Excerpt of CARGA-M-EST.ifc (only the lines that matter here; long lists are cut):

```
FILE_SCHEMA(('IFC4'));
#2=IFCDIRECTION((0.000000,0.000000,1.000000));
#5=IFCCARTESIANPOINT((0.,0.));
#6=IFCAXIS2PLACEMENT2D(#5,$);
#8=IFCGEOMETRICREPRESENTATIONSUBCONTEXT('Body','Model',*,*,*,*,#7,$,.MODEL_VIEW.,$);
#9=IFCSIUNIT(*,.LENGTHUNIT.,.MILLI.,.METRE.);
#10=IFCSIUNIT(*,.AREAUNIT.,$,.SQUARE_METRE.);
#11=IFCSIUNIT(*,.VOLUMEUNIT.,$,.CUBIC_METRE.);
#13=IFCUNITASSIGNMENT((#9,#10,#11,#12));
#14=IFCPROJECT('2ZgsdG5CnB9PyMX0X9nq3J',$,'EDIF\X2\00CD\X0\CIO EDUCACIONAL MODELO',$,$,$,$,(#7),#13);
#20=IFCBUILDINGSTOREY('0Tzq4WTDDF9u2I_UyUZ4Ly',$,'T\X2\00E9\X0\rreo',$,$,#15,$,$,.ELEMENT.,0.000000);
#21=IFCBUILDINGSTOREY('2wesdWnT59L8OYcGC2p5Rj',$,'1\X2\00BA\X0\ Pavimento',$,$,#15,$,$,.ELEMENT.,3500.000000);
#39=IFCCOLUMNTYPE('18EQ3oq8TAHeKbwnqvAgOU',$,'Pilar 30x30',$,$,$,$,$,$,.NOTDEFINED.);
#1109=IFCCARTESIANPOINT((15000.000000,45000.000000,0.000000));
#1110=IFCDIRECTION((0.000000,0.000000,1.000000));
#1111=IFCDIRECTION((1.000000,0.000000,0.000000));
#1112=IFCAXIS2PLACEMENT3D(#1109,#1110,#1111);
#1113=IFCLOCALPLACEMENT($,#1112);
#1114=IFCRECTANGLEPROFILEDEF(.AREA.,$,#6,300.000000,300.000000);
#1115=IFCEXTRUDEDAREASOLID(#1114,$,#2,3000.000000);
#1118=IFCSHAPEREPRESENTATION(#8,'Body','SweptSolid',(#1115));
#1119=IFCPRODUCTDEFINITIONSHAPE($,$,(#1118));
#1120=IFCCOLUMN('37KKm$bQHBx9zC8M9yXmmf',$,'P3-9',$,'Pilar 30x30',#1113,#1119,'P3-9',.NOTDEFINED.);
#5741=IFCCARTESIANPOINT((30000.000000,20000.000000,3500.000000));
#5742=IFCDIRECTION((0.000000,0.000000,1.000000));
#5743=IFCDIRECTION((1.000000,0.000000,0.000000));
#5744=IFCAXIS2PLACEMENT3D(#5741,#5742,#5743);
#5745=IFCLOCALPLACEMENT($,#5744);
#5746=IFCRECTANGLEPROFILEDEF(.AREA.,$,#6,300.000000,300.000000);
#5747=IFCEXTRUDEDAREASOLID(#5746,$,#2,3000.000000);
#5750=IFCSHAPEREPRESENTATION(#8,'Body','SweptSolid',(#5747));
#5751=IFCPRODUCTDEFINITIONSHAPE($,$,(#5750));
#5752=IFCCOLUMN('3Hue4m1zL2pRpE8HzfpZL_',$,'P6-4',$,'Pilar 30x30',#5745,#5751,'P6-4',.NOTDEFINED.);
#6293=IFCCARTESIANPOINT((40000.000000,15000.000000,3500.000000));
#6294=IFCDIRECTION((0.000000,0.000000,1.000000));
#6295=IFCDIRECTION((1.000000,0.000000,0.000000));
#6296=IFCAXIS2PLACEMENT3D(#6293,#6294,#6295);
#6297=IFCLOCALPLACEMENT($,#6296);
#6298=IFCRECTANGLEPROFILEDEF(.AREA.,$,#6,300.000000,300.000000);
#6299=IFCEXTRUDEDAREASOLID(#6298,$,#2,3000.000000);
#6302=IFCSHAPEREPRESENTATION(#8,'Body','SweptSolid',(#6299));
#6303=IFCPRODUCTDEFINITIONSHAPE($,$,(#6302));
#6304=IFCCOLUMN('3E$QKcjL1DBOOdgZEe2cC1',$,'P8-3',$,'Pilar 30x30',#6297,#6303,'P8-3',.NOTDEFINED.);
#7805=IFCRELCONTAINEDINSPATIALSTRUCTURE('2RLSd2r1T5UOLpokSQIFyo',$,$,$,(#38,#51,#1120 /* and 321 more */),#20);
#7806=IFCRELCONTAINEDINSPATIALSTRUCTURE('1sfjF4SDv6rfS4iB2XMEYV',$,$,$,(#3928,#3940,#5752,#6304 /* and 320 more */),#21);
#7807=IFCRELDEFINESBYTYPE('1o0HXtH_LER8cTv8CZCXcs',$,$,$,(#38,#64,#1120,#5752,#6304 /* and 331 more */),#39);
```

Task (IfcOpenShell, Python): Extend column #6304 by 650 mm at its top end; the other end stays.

```python
import ifcopenshell
import ifcopenshell.util.representation

model = ifcopenshell.open("CARGA-M-EST.ifc")

member = model.by_guid("3E$QKcjL1DBOOdgZEe2cC1")
change = 650.0

# The extrusion runs towards the end named, so only its depth changes.
body = ifcopenshell.util.representation.get_representation(member, "Model", "Body")
solid = body.Items[0]
old_length = solid.Depth
solid.Depth += change

print(f"length {old_length:g} -> {solid.Depth:g}")

model.write("CARGA-M-EST_v2.ifc")
```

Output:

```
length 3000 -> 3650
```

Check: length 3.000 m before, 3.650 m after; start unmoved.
